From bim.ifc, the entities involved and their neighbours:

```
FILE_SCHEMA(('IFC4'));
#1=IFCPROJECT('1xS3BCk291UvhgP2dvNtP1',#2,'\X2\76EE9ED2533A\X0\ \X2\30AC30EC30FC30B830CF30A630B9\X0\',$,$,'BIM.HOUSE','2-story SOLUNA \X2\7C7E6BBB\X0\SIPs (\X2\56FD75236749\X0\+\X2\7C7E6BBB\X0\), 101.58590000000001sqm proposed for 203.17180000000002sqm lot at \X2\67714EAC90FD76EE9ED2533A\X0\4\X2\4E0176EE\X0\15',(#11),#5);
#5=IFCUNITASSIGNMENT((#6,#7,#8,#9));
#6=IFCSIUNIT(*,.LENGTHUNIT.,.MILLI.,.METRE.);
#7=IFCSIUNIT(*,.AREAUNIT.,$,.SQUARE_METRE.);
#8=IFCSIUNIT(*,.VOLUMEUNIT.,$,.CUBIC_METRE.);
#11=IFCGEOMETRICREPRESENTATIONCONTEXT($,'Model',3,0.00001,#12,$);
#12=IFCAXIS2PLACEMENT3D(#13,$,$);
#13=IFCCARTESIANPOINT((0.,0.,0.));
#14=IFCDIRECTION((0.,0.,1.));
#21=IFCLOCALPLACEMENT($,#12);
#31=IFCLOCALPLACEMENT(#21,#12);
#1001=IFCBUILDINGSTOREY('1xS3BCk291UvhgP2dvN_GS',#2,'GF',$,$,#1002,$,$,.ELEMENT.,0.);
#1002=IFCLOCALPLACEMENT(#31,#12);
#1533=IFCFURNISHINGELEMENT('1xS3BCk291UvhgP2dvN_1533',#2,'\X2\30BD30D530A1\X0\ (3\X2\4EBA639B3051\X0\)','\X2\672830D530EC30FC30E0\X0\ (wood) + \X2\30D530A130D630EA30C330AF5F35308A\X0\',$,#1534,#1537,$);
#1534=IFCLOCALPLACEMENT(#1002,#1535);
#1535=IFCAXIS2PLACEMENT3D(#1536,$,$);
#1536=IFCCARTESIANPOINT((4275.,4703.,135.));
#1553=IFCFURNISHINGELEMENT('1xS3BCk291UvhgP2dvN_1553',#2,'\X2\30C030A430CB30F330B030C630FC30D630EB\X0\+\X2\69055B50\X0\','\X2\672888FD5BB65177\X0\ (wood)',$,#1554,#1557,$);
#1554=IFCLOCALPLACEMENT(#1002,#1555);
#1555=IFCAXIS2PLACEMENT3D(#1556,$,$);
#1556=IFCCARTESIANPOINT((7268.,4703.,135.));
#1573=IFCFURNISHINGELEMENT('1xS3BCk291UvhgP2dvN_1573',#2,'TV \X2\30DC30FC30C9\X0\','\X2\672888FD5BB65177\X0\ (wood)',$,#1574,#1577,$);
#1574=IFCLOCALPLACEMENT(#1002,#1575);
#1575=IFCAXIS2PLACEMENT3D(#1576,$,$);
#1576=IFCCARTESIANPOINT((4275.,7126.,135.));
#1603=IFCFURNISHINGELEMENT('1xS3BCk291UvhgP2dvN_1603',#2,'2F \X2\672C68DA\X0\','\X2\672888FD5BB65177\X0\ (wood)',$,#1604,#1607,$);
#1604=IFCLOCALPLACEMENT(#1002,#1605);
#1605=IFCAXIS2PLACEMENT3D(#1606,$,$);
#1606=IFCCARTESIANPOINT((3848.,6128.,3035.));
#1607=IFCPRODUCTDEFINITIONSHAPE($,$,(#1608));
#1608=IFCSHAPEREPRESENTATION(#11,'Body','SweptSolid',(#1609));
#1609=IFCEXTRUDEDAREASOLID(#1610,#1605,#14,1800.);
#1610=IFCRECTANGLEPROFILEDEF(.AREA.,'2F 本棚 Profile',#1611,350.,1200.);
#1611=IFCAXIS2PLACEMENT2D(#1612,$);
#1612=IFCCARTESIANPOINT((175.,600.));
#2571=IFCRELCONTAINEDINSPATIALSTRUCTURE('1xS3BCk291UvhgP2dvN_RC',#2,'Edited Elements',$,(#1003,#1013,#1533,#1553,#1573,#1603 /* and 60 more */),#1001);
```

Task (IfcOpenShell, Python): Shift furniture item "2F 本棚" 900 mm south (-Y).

```python
import ifcopenshell
import ifcopenshell.api.geometry
import ifcopenshell.util.placement
import ifcopenshell.util.unit

model = ifcopenshell.open("bim.ifc")
unit_scale = ifcopenshell.util.unit.calculate_unit_scale(model)

item = model.by_guid("1xS3BCk291UvhgP2dvN_1603")
matrix = ifcopenshell.util.placement.get_local_placement(item.ObjectPlacement)
matrix[1, 3] -= 0.9 / unit_scale
ifcopenshell.api.geometry.edit_object_placement(model, product=item, matrix=matrix, is_si=False)

print(ifcopenshell.util.placement.get_local_placement(item.ObjectPlacement).round(3) + 0.0)

model.write("bim-out.ifc")
```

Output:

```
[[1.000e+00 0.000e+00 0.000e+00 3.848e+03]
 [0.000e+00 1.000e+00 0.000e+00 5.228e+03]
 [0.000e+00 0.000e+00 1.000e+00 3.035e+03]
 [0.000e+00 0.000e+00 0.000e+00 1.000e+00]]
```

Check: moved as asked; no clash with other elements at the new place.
